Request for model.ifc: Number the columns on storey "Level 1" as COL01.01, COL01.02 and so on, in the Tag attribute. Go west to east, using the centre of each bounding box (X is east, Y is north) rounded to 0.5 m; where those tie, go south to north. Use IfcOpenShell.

First a look at what the model holds.

```python
import ifcopenshell
import ifcopenshell.util.element
import ifcopenshell.util.placement

model = ifcopenshell.open("model.ifc")
print(model.schema)
storey = next(s for s in model.by_type("IfcBuildingStorey") if s.Name == "Level 1")
columns = [e for e in ifcopenshell.util.element.get_decomposition(storey) if e.is_a("IfcColumn")]
for e in sorted(columns, key=lambda e: e.id()):
    origin = ifcopenshell.util.placement.get_local_placement(e.ObjectPlacement)[:3, 3]
    print(e.id(), e.Tag, e.Name, origin.round(2) + 0.0, sep=" | ")
```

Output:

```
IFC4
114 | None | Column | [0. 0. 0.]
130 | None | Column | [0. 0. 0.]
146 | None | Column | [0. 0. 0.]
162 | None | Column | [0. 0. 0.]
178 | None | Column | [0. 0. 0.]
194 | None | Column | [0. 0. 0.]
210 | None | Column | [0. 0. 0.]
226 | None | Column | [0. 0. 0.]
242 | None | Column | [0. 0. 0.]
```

```python
import ifcopenshell
import ifcopenshell.geom
import ifcopenshell.util.element
import ifcopenshell.util.shape

model = ifcopenshell.open("model.ifc")
settings = ifcopenshell.geom.settings()
settings.set("use-world-coords", True)


def centre(element):
    shape = ifcopenshell.geom.create_shape(settings, element)
    return ifcopenshell.util.shape.get_bbox_centroid(shape.geometry)


storey = next(s for s in model.by_type("IfcBuildingStorey") if s.Name == "Level 1")
columns = [e for e in ifcopenshell.util.element.get_decomposition(storey) if e.is_a("IfcColumn")]

# Insertion points can sit at a corner or the storey origin, so sort by the geometry (in metres).
centres = {e: centre(e) for e in columns}
columns.sort(key=lambda e: (round(centres[e][0] / 0.5), centres[e][1]))

for i, e in enumerate(columns, start=1):
    number = f"COL01.{i:02d}"
    e.Tag = number
    print(e.id(), number)

model.write("model_updated.ifc")
```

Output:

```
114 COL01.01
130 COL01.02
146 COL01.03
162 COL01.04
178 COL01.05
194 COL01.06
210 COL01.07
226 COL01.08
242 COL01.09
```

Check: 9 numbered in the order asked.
